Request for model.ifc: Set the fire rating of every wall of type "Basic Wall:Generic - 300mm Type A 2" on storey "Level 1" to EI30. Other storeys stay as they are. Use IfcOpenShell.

First a look at what the model holds.

```python
import ifcopenshell
import ifcopenshell.util.element

model = ifcopenshell.open("model.ifc")
print(model.schema)
storey = next(s for s in model.by_type("IfcBuildingStorey") if s.Name == "Level 1")
walls = [e for e in ifcopenshell.util.element.get_decomposition(storey) if e.is_a("IfcWall")]
seen = {}
for e in walls:
    element_type = ifcopenshell.util.element.get_type(e)
    key = (element_type.Name if element_type != e and element_type else None, ifcopenshell.util.element.get_pset(e, "Pset_WallCommon", "FireRating"))
    seen[key] = seen.get(key, 0) + 1
for (name, value), count in sorted(seen.items(), key=str):
    print(count, "x", name, "|", value)
```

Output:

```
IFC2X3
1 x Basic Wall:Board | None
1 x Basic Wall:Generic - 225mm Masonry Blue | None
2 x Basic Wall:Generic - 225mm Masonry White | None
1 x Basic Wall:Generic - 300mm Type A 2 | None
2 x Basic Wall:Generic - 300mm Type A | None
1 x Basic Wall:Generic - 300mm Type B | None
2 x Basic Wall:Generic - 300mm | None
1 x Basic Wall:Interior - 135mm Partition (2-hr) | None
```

```python
import ifcopenshell
import ifcopenshell.api.pset
import ifcopenshell.util.element

model = ifcopenshell.open("model.ifc")

storey = next(s for s in model.by_type("IfcBuildingStorey") if s.Name == "Level 1")
walls = [e for e in ifcopenshell.util.element.get_decomposition(storey) if e.is_a("IfcWall")]

count = 0
for e in walls:
    element_type = ifcopenshell.util.element.get_type(e)
    if element_type in (None, e) or element_type.Name != "Basic Wall:Generic - 300mm Type A 2":
        continue
    # add_pset returns the element's existing set when there is one.
    pset = ifcopenshell.api.pset.add_pset(model, product=e, name="Pset_WallCommon")
    ifcopenshell.api.pset.edit_pset(model, pset=pset, properties={"FireRating": "EI30"})
    count += 1

print(count, "walls updated")

model.write("model_edited.ifc")
```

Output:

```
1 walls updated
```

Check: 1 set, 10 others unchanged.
